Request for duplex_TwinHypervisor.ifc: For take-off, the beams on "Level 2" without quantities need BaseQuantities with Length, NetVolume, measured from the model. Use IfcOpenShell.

First a look at what the model holds.

```python
import ifcopenshell
import ifcopenshell.util.element
import ifcopenshell.util.unit

model = ifcopenshell.open("duplex_TwinHypervisor.ifc")
print(model.schema)
for unit_type in ("LENGTHUNIT", "AREAUNIT", "VOLUMEUNIT"):
    print(unit_type, ifcopenshell.util.unit.calculate_unit_scale(model, unit_type))
storey = next(s for s in model.by_type("IfcBuildingStorey") if s.Name == "Level 2")
beams = [e for e in ifcopenshell.util.element.get_decomposition(storey) if e.is_a("IfcBeam")]
for e in sorted(beams, key=lambda e: e.id()):
    print(e.id(), e.is_a(), e.Name, list(ifcopenshell.util.element.get_psets(e, qtos_only=True)), sep=" | ")
```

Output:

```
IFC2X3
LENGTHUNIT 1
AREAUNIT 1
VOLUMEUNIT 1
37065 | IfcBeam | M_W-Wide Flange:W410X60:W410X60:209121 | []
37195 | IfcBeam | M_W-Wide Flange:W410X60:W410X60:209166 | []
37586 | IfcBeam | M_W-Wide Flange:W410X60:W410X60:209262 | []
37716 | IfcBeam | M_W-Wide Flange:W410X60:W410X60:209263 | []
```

```python
import ifcopenshell
import ifcopenshell.api.pset
import ifcopenshell.geom
import ifcopenshell.util.element
import ifcopenshell.util.shape
import ifcopenshell.util.unit

model = ifcopenshell.open("duplex_TwinHypervisor.ifc")
unit_scale = ifcopenshell.util.unit.calculate_unit_scale(model)
volume_scale = ifcopenshell.util.unit.calculate_unit_scale(model, "VOLUMEUNIT")
settings = ifcopenshell.geom.settings()

storey = next(s for s in model.by_type("IfcBuildingStorey") if s.Name == "Level 2")
beams = [e for e in ifcopenshell.util.element.get_decomposition(storey) if e.is_a("IfcBeam")]

for e in sorted(beams, key=lambda e: e.id()):
    if ifcopenshell.util.element.get_psets(e, qtos_only=True, should_inherit=False):
        continue
    # Geometry comes back in metres, in the element's own axes.
    shape = ifcopenshell.geom.create_shape(settings, e)
    values = {
        "Length": ifcopenshell.util.shape.get_max_xyz(shape.geometry) / unit_scale,
        "NetVolume": ifcopenshell.util.shape.get_volume(shape.geometry) / volume_scale,
    }
    qto = ifcopenshell.api.pset.add_qto(model, product=e, name="BaseQuantities")
    ifcopenshell.api.pset.edit_qto(model, qto=qto, properties=values)
    print(e.id(), {k: round(v, 3) for k, v in values.items()})

model.write("duplex_TwinHypervisor_rev.ifc")
```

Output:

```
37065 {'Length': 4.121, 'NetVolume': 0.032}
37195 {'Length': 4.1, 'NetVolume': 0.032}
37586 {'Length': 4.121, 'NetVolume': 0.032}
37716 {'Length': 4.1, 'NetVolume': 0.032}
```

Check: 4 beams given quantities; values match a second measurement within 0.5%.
